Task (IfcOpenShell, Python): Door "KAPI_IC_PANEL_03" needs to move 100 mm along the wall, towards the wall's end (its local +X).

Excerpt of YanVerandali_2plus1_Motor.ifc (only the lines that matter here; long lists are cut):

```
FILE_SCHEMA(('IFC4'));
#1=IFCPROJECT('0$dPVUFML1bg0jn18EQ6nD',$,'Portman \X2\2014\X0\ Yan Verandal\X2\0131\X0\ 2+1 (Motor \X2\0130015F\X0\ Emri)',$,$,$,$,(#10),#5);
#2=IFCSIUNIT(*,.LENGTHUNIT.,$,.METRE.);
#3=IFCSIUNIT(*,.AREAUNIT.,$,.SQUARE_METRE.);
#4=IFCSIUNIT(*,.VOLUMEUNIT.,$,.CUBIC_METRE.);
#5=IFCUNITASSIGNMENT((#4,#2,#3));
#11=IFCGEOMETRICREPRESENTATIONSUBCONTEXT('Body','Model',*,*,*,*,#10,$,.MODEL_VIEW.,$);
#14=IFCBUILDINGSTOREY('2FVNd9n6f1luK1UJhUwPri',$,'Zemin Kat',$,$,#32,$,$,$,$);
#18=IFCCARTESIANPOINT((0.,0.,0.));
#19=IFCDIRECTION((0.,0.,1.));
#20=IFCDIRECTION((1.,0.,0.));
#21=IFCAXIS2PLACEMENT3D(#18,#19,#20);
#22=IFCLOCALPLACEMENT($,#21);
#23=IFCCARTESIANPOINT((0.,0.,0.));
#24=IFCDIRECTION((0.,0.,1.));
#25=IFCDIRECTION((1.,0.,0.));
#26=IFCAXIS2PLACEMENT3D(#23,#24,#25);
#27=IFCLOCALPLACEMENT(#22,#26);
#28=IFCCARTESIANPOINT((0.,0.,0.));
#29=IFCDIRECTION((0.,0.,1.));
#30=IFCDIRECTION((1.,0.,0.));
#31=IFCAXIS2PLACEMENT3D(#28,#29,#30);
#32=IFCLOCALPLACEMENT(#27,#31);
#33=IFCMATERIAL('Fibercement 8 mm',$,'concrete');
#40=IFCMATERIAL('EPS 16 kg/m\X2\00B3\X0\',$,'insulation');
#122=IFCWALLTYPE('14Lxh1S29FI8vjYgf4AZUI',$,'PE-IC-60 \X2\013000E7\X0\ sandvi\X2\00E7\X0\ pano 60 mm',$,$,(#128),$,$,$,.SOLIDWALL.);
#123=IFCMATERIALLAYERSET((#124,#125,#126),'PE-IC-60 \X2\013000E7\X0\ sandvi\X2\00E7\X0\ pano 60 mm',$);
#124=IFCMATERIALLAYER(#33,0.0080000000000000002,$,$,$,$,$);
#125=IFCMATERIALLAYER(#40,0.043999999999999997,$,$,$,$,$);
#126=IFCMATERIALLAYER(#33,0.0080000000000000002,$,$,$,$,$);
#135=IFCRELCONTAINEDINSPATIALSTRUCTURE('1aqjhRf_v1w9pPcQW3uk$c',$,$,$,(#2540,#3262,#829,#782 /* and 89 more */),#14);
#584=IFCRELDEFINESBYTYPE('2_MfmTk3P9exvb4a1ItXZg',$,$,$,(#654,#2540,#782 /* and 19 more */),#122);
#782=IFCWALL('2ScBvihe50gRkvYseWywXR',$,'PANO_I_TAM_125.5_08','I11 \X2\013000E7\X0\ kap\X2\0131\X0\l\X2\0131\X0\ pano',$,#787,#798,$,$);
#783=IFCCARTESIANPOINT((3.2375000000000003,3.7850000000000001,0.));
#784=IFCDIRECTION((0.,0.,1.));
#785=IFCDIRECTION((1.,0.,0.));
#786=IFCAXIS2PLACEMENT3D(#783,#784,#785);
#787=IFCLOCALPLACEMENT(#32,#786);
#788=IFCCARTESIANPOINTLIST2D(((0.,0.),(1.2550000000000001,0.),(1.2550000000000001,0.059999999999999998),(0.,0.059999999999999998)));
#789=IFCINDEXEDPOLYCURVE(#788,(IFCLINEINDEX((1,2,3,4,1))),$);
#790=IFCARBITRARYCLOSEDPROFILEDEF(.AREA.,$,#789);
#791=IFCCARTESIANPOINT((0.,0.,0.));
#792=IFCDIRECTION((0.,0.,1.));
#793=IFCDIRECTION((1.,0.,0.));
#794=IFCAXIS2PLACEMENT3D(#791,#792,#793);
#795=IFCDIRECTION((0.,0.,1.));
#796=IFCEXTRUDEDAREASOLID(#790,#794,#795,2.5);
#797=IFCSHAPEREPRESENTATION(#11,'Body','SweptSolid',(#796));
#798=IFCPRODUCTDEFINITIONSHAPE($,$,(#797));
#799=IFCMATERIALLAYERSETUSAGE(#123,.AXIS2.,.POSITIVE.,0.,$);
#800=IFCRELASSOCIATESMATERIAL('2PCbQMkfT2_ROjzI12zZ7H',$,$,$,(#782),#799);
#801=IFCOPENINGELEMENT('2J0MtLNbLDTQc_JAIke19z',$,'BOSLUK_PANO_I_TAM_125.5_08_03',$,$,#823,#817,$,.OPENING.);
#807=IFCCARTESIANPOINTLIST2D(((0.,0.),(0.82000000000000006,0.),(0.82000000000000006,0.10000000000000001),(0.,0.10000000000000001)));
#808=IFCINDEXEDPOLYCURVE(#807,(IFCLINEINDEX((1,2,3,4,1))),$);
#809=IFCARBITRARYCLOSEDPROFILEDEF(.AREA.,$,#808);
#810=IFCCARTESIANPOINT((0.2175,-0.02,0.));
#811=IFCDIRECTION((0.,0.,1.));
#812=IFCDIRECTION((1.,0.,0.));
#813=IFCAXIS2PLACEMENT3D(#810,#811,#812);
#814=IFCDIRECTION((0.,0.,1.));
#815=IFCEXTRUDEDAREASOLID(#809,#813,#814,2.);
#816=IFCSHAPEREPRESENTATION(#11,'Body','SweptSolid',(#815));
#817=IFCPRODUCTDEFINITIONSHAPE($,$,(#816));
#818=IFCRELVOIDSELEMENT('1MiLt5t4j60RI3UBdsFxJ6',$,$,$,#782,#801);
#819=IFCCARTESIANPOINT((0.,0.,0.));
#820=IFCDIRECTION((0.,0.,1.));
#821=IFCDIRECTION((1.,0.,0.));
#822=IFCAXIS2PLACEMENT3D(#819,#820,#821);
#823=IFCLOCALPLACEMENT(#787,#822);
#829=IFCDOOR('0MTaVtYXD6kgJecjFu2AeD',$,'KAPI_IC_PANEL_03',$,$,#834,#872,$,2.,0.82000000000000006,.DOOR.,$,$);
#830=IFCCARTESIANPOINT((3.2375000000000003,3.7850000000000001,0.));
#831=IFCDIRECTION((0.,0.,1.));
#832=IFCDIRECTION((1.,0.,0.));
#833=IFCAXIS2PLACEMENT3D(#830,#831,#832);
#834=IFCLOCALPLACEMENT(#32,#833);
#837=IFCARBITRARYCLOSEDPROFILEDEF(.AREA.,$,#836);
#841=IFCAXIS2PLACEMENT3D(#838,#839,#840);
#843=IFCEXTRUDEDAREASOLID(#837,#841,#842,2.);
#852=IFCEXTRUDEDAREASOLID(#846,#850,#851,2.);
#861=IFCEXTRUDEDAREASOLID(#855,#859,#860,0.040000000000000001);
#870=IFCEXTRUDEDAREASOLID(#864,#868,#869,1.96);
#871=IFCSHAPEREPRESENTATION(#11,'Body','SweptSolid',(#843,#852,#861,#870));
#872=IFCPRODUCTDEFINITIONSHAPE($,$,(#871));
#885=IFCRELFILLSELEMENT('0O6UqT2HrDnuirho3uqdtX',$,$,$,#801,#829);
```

```python
import ifcopenshell
import ifcopenshell.api.geometry
import ifcopenshell.util.placement
import ifcopenshell.util.unit

model = ifcopenshell.open("YanVerandali_2plus1_Motor.ifc")
unit_scale = ifcopenshell.util.unit.calculate_unit_scale(model)

door = model.by_guid("0MTaVtYXD6kgJecjFu2AeD")
opening = door.FillsVoids[0].RelatingOpeningElement
wall = opening.VoidsElements[0].RelatingBuildingElement

wall_matrix = ifcopenshell.util.placement.get_local_placement(wall.ObjectPlacement)
shift = wall_matrix[:3, 0] * 0.1 / unit_scale
before = ifcopenshell.util.placement.get_local_placement(door.ObjectPlacement)[:3, 3].copy()

# The door is not placed relative to its opening, so move both.
for product in (opening, door):
    matrix = ifcopenshell.util.placement.get_local_placement(product.ObjectPlacement)
    matrix[:3, 3] += shift
    ifcopenshell.api.geometry.edit_object_placement(model, product=product, matrix=matrix, is_si=False)

after = ifcopenshell.util.placement.get_local_placement(door.ObjectPlacement)[:3, 3]
print("door moved by", (after - before).round(3) + 0.0)

model.write("YanVerandali_2plus1_Motor_edited.ifc")
```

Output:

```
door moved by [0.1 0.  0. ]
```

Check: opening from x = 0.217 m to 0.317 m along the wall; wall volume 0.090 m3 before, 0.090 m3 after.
